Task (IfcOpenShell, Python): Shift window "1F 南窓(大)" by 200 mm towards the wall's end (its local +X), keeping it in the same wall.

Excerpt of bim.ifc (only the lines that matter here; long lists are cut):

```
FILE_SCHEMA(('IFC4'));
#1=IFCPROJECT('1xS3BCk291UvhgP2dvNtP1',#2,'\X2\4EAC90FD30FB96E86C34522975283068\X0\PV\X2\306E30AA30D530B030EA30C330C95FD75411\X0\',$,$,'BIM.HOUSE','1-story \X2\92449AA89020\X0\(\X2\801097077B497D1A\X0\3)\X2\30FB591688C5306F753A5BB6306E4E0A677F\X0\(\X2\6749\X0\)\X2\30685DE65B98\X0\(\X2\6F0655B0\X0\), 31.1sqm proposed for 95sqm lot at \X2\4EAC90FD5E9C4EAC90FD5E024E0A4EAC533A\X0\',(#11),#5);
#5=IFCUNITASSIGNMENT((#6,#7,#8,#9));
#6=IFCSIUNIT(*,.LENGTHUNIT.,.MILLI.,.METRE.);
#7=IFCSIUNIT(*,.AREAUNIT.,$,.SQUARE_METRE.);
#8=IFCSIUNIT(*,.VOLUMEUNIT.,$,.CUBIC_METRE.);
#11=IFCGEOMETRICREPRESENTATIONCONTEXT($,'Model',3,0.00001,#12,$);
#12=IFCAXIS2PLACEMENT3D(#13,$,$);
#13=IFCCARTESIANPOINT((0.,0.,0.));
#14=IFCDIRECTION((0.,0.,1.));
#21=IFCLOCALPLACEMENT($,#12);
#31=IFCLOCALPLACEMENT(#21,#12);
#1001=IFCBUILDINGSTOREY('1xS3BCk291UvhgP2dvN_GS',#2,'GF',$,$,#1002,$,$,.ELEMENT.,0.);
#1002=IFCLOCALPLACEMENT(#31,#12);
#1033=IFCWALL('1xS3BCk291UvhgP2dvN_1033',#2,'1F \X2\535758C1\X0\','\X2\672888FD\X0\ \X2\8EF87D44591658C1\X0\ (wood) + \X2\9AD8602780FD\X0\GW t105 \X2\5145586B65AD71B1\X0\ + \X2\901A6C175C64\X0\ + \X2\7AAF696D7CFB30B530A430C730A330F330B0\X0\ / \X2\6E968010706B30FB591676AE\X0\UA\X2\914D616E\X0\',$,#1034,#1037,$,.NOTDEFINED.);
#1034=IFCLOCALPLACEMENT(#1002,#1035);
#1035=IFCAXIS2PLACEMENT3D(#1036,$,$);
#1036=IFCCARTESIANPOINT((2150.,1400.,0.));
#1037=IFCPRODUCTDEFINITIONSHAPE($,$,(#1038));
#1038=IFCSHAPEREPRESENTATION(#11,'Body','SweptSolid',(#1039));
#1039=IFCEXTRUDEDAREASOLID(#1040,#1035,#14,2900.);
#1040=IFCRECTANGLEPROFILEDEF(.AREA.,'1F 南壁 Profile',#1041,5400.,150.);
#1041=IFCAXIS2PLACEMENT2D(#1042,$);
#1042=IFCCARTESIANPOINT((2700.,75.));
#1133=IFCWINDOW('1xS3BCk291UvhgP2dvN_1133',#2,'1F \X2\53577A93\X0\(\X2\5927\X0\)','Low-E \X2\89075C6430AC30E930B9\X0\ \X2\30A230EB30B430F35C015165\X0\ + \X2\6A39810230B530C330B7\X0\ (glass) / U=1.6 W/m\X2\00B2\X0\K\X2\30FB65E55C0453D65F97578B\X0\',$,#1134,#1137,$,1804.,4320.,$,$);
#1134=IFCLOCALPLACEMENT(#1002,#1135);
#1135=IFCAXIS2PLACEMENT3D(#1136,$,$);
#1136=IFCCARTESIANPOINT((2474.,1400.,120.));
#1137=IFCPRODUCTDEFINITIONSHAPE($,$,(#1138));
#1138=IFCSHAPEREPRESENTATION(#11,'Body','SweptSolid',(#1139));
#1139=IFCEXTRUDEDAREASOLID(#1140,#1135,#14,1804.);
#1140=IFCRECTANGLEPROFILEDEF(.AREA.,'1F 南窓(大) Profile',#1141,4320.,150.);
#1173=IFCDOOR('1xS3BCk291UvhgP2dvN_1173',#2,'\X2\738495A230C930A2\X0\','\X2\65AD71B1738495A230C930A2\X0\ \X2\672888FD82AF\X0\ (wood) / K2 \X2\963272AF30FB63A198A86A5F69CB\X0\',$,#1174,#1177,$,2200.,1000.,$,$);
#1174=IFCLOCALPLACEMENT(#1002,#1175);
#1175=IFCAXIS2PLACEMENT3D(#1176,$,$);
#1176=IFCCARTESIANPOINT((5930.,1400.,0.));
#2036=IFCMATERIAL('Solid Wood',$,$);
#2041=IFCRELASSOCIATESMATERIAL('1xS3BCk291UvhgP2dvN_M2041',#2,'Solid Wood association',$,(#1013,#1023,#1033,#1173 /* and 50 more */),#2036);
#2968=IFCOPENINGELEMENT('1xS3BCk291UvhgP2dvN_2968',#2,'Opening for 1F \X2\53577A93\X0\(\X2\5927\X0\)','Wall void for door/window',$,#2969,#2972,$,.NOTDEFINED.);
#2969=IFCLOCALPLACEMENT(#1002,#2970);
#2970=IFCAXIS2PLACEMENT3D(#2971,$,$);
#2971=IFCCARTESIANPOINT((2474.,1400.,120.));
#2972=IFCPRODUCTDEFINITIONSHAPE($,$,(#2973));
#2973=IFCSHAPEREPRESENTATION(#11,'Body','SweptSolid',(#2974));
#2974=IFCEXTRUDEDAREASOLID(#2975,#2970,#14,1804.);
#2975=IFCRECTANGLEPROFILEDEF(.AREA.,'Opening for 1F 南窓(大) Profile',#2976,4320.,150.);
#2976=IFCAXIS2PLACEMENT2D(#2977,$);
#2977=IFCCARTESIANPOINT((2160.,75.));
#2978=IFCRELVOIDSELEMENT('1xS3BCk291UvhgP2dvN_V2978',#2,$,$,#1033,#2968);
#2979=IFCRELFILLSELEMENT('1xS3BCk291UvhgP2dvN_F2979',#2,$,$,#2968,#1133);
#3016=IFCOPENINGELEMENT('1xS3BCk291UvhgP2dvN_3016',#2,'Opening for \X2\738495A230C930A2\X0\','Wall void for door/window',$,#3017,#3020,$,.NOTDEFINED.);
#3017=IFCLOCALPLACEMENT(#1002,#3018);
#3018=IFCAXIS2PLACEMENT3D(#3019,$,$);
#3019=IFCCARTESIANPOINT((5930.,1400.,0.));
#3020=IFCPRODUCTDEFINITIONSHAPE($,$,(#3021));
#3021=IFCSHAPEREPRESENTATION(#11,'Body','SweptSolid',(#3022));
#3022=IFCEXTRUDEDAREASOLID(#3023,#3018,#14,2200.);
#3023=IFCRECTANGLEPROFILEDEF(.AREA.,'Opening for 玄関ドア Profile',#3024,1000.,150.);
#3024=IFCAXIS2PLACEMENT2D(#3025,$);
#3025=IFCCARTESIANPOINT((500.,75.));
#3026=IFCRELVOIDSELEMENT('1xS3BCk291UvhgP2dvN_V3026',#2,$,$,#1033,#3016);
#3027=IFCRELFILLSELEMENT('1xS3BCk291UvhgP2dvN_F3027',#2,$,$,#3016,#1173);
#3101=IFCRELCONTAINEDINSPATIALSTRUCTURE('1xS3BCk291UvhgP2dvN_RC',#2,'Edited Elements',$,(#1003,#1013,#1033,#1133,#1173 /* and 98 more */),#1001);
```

```python
import ifcopenshell
import ifcopenshell.api.geometry
import ifcopenshell.util.placement
import ifcopenshell.util.unit

model = ifcopenshell.open("bim.ifc")
unit_scale = ifcopenshell.util.unit.calculate_unit_scale(model)

window = model.by_id(1133)
opening = window.FillsVoids[0].RelatingOpeningElement
wall = opening.VoidsElements[0].RelatingBuildingElement

wall_matrix = ifcopenshell.util.placement.get_local_placement(wall.ObjectPlacement)
shift = wall_matrix[:3, 0] * 0.2 / unit_scale
before = ifcopenshell.util.placement.get_local_placement(window.ObjectPlacement)[:3, 3].copy()

# The window is not placed relative to its opening, so move both.
for product in (opening, window):
    matrix = ifcopenshell.util.placement.get_local_placement(product.ObjectPlacement)
    matrix[:3, 3] += shift
    ifcopenshell.api.geometry.edit_object_placement(model, product=product, matrix=matrix, is_si=False)

after = ifcopenshell.util.placement.get_local_placement(window.ObjectPlacement)[:3, 3]
print("window moved by", (after - before).round(3) + 0.0)

model.write("bim_edited.ifc")
```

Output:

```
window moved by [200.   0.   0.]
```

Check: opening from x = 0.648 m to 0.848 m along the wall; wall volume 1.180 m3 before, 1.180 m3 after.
